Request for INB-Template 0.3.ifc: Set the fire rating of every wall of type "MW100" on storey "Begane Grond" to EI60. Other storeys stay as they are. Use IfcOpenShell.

First a look at what the model holds.

```python
import ifcopenshell
import ifcopenshell.util.element

model = ifcopenshell.open("INB-Template 0.3.ifc")
print(model.schema)
storey = next(s for s in model.by_type("IfcBuildingStorey") if s.Name == "Begane Grond")
walls = [e for e in ifcopenshell.util.element.get_decomposition(storey) if e.is_a("IfcWall")]
seen = {}
for e in walls:
    element_type = ifcopenshell.util.element.get_type(e)
    key = (element_type.Name if element_type != e and element_type else None, ifcopenshell.util.element.get_pset(e, "Pset_WallCommon", "FireRating"))
    seen[key] = seen.get(key, 0) + 1
for (name, value), count in sorted(seen.items(), key=str):
    print(count, "x", name, "|", value)
```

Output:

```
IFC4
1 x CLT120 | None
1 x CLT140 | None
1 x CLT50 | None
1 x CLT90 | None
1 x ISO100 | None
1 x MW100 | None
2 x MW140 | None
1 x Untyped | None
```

```python
import ifcopenshell
import ifcopenshell.api.pset
import ifcopenshell.util.element

model = ifcopenshell.open("INB-Template 0.3.ifc")

storey = next(s for s in model.by_type("IfcBuildingStorey") if s.Name == "Begane Grond")
walls = [e for e in ifcopenshell.util.element.get_decomposition(storey) if e.is_a("IfcWall")]

count = 0
for e in walls:
    element_type = ifcopenshell.util.element.get_type(e)
    if element_type in (None, e) or element_type.Name != "MW100":
        continue
    # add_pset returns the element's existing set when there is one.
    pset = ifcopenshell.api.pset.add_pset(model, product=e, name="Pset_WallCommon")
    ifcopenshell.api.pset.edit_pset(model, pset=pset, properties={"FireRating": "EI60"})
    count += 1

print(count, "walls updated")

model.write("INB-Template 0.3-out.ifc")
```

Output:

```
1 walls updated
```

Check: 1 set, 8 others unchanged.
